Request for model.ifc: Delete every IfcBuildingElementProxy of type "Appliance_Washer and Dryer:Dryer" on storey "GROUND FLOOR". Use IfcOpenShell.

First a look at what the model holds.

```python
import ifcopenshell
import ifcopenshell.util.element

model = ifcopenshell.open("model.ifc")
print(model.schema)
storey = next(s for s in model.by_type("IfcBuildingStorey") if s.Name == "GROUND FLOOR")
proxies = [e for e in ifcopenshell.util.element.get_decomposition(storey) if e.is_a("IfcBuildingElementProxy")]
seen = {}
for e in proxies:
    element_type = ifcopenshell.util.element.get_type(e)
    name = element_type.Name if element_type not in (None, e) else None
    seen[name] = seen.get(name, 0) + 1
for name, count in sorted(seen.items(), key=str):
    print(count, "x", name)
```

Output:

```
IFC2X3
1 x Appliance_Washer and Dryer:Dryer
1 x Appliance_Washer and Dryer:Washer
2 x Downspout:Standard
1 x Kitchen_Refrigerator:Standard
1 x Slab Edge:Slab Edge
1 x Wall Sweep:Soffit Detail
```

```python
import ifcopenshell
import ifcopenshell.api.root
import ifcopenshell.util.element

model = ifcopenshell.open("model.ifc")

storey = next(s for s in model.by_type("IfcBuildingStorey") if s.Name == "GROUND FLOOR")
proxies = [e for e in ifcopenshell.util.element.get_decomposition(storey) if e.is_a("IfcBuildingElementProxy")]
targets = [e for e in proxies if (t := ifcopenshell.util.element.get_type(e)) not in (None, e) and t.Name == "Appliance_Washer and Dryer:Dryer"]

for e in targets:
    ifcopenshell.api.root.remove_product(model, product=e)
print(len(targets), "removed")

model.write("model_edited.ifc")
```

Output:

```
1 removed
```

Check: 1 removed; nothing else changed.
